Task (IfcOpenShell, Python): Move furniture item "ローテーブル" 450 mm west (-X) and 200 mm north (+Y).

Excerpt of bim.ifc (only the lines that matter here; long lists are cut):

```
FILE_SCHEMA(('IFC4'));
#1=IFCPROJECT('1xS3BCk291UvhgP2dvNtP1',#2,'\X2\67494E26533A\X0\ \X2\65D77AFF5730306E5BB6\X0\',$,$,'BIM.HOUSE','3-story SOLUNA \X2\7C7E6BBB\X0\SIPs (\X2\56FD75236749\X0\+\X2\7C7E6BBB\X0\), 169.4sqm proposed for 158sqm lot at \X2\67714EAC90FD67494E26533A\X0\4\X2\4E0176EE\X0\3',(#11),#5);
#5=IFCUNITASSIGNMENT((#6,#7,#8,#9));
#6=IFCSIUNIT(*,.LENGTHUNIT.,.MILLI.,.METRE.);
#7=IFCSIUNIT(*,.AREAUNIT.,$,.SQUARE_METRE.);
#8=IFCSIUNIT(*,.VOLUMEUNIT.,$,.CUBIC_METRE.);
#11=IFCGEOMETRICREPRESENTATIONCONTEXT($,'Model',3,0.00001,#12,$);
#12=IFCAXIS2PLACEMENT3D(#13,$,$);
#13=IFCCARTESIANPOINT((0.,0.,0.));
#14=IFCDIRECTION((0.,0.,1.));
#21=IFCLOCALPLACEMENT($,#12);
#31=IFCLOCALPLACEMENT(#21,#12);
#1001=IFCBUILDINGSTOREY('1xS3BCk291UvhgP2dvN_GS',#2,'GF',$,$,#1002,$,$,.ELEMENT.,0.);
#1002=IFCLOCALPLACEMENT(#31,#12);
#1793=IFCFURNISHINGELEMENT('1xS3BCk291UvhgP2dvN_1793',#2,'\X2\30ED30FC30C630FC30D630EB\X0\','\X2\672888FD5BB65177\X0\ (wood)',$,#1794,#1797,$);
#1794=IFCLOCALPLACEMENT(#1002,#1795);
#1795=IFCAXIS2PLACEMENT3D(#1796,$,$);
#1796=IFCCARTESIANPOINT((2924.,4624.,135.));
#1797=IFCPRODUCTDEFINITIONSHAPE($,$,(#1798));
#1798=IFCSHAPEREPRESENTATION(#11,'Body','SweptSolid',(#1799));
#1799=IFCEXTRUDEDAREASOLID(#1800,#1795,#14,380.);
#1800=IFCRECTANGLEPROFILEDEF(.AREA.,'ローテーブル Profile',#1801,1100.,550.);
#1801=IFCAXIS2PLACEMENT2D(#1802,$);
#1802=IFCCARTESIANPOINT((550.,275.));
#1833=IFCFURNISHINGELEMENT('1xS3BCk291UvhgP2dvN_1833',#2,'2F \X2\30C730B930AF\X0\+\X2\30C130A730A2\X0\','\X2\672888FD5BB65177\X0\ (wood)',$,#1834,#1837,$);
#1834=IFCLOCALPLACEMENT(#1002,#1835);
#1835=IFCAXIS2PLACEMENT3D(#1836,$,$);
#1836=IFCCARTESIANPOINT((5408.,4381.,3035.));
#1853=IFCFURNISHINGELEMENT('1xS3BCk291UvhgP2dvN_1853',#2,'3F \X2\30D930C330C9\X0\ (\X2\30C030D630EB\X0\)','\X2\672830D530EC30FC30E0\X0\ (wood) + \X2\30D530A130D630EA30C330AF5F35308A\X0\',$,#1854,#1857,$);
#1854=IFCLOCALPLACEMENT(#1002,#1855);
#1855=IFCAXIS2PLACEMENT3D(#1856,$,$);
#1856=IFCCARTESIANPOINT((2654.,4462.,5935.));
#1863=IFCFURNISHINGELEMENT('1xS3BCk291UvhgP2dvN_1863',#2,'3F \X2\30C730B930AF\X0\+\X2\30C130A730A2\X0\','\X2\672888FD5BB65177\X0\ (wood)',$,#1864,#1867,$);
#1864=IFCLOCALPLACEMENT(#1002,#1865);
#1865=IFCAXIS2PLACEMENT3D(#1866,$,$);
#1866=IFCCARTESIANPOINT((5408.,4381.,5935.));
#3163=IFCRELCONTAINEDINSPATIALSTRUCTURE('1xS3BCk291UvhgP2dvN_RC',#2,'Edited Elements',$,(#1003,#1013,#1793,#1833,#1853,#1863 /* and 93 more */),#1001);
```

```python
import ifcopenshell
import ifcopenshell.api.geometry
import ifcopenshell.util.placement

model = ifcopenshell.open("bim.ifc")

item = model.by_guid("1xS3BCk291UvhgP2dvN_1793")
matrix = ifcopenshell.util.placement.get_local_placement(item.ObjectPlacement)
matrix[0, 3] -= 450.0
matrix[1, 3] += 200.0
ifcopenshell.api.geometry.edit_object_placement(model, product=item, matrix=matrix, is_si=False)

print(ifcopenshell.util.placement.get_local_placement(item.ObjectPlacement).round(3) + 0.0)

model.write("bim_rev.ifc")
```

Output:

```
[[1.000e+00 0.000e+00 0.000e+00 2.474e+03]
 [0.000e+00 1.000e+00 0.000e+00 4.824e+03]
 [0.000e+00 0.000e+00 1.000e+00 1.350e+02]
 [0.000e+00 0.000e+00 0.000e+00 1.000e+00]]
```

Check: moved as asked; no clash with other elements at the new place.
